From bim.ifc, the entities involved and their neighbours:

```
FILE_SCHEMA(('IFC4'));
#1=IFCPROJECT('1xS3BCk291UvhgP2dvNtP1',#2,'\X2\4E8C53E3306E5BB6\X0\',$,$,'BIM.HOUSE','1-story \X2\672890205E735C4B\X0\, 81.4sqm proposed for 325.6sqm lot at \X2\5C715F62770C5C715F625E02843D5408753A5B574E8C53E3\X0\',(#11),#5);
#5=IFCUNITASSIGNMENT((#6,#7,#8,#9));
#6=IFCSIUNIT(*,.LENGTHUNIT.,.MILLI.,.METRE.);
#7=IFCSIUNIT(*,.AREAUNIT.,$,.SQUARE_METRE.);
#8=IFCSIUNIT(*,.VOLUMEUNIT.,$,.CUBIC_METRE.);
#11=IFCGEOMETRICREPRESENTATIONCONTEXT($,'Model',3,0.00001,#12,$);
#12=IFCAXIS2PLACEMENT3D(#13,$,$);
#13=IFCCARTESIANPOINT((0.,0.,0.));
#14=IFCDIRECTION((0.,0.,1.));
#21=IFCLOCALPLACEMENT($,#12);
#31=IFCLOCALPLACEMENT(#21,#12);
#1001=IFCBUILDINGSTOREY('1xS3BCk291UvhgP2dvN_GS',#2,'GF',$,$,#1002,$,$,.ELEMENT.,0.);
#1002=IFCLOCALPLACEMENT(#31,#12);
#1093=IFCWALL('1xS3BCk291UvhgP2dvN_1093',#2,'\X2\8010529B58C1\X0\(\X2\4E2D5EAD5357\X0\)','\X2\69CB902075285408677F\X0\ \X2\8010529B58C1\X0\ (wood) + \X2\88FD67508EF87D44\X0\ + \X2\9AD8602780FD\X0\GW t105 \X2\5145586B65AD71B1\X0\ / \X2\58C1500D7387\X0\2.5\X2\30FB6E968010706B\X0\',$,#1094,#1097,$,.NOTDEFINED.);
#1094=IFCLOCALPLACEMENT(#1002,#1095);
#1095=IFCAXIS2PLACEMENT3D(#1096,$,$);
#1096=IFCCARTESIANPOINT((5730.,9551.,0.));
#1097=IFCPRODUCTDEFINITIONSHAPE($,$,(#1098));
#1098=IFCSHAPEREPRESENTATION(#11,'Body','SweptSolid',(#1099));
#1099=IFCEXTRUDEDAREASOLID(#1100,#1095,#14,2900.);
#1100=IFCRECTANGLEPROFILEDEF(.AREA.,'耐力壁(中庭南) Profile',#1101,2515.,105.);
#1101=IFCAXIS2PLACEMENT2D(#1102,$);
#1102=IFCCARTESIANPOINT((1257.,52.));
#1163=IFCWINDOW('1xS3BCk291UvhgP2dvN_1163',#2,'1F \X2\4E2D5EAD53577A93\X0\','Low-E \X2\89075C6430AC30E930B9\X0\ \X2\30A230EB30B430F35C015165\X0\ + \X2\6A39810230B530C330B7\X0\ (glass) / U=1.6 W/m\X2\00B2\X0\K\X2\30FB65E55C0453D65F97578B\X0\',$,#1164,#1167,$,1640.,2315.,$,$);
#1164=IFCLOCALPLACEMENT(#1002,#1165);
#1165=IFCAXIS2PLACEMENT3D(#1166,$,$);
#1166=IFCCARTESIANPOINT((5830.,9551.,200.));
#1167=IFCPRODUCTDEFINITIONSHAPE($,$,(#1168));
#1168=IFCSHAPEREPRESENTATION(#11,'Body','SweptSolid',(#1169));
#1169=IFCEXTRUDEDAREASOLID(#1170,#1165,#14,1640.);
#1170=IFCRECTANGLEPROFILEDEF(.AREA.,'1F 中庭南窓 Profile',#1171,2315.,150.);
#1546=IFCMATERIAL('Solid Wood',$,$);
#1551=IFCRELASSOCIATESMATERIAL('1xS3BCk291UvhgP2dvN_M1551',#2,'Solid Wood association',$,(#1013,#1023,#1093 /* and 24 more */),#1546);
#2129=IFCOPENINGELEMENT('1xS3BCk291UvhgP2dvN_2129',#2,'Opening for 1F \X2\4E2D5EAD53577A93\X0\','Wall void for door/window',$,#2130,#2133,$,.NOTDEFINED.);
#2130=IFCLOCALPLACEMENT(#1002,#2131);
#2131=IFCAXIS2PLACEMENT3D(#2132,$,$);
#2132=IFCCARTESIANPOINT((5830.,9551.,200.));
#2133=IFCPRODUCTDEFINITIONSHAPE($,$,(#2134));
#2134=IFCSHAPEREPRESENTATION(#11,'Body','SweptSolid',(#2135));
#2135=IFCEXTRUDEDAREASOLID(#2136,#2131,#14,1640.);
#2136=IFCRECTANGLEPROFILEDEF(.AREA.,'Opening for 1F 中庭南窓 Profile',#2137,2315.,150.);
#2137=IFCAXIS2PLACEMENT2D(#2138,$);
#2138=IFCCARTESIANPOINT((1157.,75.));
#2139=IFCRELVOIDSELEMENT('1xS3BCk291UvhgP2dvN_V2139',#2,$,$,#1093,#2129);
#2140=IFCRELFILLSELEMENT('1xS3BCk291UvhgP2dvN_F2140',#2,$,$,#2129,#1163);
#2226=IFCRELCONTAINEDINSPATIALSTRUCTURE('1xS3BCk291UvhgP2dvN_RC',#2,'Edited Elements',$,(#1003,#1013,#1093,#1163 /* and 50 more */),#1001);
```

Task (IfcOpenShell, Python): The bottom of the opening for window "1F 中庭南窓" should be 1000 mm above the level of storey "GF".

```python
import numpy as np
import ifcopenshell
import ifcopenshell.api.geometry
import ifcopenshell.geom
import ifcopenshell.util.element
import ifcopenshell.util.placement
import ifcopenshell.util.shape
import ifcopenshell.util.unit

model = ifcopenshell.open("bim.ifc")
unit_scale = ifcopenshell.util.unit.calculate_unit_scale(model)

window = model.by_id(1163)
opening = window.FillsVoids[0].RelatingOpeningElement
storey = ifcopenshell.util.element.get_container(window, ifc_class="IfcBuildingStorey")
level = ifcopenshell.util.placement.get_local_placement(storey.ObjectPlacement)[2, 3]

# The opening's origin need not be at the sill, so measure its lowest point.
shape = ifcopenshell.geom.create_shape(ifcopenshell.geom.settings(), opening)
bottom = ifcopenshell.util.shape.get_shape_bottom_elevation(shape, shape.geometry) / unit_scale
dz = level + 1000.0 - bottom

shift = np.array([0.0, 0.0, dz])
# The window is not placed relative to its opening, so move both.
for product in (opening, window):
    matrix = ifcopenshell.util.placement.get_local_placement(product.ObjectPlacement)
    matrix[:3, 3] += shift
    ifcopenshell.api.geometry.edit_object_placement(model, product=product, matrix=matrix, is_si=False)

print(f"moved by {dz * unit_scale:+.3f} m")

model.write("bim-out.ifc")
```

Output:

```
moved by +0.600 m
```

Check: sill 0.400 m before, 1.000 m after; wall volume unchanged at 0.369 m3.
